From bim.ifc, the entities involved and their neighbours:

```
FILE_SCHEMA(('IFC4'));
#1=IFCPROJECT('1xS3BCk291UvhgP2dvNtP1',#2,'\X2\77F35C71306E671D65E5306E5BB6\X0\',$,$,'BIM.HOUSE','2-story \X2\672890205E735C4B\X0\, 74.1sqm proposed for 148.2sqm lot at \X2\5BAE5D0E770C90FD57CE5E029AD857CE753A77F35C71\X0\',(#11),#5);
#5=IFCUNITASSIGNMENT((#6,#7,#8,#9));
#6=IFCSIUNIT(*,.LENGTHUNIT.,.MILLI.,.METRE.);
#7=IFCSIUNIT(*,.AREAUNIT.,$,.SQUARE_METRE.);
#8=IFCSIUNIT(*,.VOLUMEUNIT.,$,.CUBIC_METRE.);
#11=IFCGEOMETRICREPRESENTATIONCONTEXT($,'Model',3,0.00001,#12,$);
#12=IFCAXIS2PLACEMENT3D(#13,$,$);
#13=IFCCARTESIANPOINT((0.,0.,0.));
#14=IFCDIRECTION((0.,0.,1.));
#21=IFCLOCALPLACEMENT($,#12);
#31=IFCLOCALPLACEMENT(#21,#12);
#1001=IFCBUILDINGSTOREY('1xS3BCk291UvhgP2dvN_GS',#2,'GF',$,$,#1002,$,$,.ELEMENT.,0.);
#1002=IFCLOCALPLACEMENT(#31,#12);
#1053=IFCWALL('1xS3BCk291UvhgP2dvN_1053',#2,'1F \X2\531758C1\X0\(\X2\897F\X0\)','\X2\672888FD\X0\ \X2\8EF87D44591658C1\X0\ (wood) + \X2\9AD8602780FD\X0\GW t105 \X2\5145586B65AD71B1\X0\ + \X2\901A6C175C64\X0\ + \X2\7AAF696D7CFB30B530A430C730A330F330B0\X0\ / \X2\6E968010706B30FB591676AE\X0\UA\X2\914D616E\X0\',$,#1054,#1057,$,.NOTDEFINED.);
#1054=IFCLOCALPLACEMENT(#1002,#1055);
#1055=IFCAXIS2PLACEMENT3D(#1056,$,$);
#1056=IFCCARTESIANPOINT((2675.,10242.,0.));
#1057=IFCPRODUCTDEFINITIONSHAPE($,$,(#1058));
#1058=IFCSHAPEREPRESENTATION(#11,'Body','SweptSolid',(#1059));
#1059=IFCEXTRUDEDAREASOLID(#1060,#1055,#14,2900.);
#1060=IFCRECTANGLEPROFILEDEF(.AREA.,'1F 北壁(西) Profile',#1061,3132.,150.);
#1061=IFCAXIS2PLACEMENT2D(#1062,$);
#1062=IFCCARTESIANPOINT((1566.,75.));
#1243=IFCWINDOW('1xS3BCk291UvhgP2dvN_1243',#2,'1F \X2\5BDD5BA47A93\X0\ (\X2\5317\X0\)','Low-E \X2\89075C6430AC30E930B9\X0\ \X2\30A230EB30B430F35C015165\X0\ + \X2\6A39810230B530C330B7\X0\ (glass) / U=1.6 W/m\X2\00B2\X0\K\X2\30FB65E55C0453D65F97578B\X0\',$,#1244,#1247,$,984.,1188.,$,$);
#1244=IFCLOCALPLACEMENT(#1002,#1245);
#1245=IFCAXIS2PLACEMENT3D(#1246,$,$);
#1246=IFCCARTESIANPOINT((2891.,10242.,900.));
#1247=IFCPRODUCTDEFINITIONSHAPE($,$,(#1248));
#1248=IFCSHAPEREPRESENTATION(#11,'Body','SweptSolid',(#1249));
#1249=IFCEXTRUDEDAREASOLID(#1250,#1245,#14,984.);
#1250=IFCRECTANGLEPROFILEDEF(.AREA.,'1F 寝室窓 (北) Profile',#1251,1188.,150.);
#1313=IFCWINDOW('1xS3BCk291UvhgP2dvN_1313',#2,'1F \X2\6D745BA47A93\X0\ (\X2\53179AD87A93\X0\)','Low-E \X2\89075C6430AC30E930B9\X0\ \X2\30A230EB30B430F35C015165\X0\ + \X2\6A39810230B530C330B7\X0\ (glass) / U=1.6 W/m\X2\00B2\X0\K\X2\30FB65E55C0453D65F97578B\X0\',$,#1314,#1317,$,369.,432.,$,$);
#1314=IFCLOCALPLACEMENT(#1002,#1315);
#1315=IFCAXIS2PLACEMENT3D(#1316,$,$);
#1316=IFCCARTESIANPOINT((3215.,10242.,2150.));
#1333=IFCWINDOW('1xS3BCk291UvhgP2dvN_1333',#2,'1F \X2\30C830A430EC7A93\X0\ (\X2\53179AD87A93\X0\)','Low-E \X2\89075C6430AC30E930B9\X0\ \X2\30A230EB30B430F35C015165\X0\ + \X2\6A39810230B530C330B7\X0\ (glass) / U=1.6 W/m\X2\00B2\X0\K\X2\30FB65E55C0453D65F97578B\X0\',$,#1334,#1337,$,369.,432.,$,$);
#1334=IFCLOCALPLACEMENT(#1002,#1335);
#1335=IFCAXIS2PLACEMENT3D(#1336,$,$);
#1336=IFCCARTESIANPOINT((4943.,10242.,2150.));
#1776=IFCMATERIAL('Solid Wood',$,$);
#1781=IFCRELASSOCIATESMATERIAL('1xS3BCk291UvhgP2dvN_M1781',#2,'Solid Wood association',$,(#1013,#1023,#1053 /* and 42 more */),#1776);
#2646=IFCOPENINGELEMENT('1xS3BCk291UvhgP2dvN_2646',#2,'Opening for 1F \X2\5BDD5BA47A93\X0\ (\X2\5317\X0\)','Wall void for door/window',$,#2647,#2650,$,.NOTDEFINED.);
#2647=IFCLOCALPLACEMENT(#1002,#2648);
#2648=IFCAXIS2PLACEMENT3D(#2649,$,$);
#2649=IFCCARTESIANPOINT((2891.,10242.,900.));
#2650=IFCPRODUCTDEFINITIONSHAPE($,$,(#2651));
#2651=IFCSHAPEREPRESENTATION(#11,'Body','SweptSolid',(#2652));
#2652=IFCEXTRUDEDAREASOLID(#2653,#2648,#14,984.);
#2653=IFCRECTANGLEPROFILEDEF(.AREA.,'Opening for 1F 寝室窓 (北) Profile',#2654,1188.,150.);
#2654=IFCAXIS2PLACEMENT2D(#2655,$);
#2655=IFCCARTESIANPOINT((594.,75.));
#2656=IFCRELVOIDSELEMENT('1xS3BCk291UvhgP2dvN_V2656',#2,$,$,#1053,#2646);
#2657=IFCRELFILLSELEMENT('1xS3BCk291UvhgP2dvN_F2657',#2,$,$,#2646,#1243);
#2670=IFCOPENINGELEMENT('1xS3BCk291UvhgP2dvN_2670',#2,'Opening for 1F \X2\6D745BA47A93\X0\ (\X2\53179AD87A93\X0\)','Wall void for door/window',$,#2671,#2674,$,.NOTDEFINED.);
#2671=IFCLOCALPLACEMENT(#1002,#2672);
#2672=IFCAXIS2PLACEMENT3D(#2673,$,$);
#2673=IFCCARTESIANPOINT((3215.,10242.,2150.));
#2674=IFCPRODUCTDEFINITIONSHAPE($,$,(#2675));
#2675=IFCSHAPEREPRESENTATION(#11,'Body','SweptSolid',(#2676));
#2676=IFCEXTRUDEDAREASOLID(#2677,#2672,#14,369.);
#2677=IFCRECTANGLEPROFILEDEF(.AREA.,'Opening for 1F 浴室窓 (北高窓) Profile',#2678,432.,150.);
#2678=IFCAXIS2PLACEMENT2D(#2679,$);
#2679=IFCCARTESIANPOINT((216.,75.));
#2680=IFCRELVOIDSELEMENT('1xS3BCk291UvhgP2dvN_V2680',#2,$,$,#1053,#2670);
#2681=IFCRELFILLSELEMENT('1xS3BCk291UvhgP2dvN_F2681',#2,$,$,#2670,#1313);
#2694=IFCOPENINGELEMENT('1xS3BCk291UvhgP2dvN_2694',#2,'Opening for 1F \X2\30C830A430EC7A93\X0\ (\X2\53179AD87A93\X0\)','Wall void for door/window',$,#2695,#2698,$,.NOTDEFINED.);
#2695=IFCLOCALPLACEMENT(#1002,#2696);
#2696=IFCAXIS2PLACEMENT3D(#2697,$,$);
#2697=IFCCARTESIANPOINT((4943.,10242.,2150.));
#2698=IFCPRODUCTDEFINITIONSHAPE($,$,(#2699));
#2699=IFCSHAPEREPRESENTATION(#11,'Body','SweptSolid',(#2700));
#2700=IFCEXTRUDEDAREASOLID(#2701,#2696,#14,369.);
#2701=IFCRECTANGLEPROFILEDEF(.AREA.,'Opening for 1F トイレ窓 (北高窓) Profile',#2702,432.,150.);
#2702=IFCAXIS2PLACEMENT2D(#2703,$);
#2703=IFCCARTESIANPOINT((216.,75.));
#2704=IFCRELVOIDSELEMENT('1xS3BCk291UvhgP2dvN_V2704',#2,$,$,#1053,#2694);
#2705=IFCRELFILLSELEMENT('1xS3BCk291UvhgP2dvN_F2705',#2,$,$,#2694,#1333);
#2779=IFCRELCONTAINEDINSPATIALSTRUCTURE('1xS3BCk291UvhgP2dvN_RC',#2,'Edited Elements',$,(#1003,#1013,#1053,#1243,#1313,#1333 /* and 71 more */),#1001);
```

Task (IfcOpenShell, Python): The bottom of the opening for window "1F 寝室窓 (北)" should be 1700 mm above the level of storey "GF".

```python
import numpy as np
import ifcopenshell
import ifcopenshell.api.geometry
import ifcopenshell.geom
import ifcopenshell.util.element
import ifcopenshell.util.placement
import ifcopenshell.util.shape
import ifcopenshell.util.unit

model = ifcopenshell.open("bim.ifc")
unit_scale = ifcopenshell.util.unit.calculate_unit_scale(model)

window = model.by_guid("1xS3BCk291UvhgP2dvN_1243")
opening = window.FillsVoids[0].RelatingOpeningElement
storey = ifcopenshell.util.element.get_container(window, ifc_class="IfcBuildingStorey")
level = ifcopenshell.util.placement.get_local_placement(storey.ObjectPlacement)[2, 3]

# The opening's origin need not be at the sill, so measure its lowest point.
shape = ifcopenshell.geom.create_shape(ifcopenshell.geom.settings(), opening)
bottom = ifcopenshell.util.shape.get_shape_bottom_elevation(shape, shape.geometry) / unit_scale
dz = level + 1700.0 - bottom

shift = np.array([0.0, 0.0, dz])
# The window is not placed relative to its opening, so move both.
for product in (opening, window):
    matrix = ifcopenshell.util.placement.get_local_placement(product.ObjectPlacement)
    matrix[:3, 3] += shift
    ifcopenshell.api.geometry.edit_object_placement(model, product=product, matrix=matrix, is_si=False)

print(f"moved by {dz * unit_scale:+.3f} m")

model.write("bim_edited.ifc")
```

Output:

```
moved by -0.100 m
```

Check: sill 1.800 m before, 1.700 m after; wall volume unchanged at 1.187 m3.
